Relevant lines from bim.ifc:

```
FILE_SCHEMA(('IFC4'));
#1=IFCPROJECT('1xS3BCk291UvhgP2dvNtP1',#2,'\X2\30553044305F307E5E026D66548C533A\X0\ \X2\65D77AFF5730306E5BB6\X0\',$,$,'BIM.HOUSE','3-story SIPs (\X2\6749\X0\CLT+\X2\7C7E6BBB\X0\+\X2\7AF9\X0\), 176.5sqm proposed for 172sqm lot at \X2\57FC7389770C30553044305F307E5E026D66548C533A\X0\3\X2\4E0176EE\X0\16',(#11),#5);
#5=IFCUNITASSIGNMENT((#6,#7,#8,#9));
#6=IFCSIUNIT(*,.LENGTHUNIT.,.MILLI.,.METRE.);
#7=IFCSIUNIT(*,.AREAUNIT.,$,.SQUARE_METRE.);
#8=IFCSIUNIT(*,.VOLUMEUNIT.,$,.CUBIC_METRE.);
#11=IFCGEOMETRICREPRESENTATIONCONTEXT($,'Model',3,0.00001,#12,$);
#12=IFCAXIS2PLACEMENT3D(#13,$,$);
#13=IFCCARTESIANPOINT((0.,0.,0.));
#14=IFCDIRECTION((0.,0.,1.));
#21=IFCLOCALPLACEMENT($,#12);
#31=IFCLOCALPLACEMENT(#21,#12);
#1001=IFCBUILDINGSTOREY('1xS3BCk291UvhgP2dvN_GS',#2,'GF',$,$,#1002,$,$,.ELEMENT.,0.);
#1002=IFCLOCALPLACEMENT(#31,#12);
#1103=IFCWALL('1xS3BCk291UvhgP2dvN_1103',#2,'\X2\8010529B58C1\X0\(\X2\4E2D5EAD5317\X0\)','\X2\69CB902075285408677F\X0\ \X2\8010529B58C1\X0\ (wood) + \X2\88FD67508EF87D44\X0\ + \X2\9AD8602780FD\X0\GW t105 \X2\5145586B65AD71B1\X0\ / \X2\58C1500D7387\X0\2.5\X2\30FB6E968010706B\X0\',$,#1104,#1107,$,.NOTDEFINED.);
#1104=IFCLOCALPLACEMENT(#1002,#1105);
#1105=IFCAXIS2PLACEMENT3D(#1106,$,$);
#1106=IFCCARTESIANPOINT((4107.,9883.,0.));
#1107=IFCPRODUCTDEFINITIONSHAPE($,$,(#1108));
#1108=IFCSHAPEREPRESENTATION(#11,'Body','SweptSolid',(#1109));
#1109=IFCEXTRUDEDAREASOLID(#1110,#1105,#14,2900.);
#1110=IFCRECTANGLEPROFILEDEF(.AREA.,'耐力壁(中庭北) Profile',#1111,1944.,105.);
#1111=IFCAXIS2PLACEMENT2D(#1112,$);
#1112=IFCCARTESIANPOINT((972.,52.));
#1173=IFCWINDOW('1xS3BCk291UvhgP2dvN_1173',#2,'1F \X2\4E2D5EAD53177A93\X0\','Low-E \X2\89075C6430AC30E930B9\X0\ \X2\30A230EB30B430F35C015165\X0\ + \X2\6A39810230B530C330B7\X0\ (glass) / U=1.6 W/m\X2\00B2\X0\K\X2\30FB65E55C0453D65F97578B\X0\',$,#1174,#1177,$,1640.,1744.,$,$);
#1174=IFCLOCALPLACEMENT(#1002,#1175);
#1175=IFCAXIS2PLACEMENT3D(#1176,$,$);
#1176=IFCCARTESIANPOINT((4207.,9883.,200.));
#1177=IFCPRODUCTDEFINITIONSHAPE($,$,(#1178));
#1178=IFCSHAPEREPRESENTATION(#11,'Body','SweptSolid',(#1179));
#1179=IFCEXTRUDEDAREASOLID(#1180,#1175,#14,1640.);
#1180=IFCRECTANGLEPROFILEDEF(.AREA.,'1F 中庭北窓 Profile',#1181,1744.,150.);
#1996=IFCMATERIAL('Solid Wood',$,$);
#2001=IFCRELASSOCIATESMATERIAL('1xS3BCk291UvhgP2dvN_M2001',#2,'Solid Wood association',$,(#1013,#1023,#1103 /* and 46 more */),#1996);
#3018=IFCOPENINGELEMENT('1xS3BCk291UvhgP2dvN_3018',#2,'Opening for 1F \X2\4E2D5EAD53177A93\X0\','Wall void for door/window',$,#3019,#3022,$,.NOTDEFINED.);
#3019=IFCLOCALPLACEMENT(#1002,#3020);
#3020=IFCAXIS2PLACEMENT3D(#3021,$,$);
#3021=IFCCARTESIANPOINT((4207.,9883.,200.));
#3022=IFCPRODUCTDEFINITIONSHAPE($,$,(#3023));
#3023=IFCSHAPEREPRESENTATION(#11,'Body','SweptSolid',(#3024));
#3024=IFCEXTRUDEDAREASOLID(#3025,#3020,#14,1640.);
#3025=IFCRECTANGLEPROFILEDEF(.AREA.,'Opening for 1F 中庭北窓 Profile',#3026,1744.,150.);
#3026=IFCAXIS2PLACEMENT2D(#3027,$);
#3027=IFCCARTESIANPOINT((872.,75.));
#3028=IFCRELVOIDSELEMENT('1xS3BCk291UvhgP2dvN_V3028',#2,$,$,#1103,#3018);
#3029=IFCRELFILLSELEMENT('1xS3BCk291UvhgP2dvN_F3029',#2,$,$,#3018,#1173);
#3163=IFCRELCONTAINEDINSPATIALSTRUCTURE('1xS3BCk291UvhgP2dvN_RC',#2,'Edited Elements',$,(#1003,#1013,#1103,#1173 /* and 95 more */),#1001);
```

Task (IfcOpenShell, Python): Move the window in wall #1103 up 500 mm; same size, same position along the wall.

```python
import numpy as np
import ifcopenshell
import ifcopenshell.api.geometry
import ifcopenshell.util.placement
import ifcopenshell.util.unit

model = ifcopenshell.open("bim.ifc")
unit_scale = ifcopenshell.util.unit.calculate_unit_scale(model)

window = model.by_guid("1xS3BCk291UvhgP2dvN_1173")
opening = window.FillsVoids[0].RelatingOpeningElement
dz = 500.0

shift = np.array([0.0, 0.0, dz])
# The window is not placed relative to its opening, so move both.
for product in (opening, window):
    matrix = ifcopenshell.util.placement.get_local_placement(product.ObjectPlacement)
    matrix[:3, 3] += shift
    ifcopenshell.api.geometry.edit_object_placement(model, product=product, matrix=matrix, is_si=False)

print(f"moved by {dz * unit_scale:+.3f} m")

model.write("bim_updated.ifc")
```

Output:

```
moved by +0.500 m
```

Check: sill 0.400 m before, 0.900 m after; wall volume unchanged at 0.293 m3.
